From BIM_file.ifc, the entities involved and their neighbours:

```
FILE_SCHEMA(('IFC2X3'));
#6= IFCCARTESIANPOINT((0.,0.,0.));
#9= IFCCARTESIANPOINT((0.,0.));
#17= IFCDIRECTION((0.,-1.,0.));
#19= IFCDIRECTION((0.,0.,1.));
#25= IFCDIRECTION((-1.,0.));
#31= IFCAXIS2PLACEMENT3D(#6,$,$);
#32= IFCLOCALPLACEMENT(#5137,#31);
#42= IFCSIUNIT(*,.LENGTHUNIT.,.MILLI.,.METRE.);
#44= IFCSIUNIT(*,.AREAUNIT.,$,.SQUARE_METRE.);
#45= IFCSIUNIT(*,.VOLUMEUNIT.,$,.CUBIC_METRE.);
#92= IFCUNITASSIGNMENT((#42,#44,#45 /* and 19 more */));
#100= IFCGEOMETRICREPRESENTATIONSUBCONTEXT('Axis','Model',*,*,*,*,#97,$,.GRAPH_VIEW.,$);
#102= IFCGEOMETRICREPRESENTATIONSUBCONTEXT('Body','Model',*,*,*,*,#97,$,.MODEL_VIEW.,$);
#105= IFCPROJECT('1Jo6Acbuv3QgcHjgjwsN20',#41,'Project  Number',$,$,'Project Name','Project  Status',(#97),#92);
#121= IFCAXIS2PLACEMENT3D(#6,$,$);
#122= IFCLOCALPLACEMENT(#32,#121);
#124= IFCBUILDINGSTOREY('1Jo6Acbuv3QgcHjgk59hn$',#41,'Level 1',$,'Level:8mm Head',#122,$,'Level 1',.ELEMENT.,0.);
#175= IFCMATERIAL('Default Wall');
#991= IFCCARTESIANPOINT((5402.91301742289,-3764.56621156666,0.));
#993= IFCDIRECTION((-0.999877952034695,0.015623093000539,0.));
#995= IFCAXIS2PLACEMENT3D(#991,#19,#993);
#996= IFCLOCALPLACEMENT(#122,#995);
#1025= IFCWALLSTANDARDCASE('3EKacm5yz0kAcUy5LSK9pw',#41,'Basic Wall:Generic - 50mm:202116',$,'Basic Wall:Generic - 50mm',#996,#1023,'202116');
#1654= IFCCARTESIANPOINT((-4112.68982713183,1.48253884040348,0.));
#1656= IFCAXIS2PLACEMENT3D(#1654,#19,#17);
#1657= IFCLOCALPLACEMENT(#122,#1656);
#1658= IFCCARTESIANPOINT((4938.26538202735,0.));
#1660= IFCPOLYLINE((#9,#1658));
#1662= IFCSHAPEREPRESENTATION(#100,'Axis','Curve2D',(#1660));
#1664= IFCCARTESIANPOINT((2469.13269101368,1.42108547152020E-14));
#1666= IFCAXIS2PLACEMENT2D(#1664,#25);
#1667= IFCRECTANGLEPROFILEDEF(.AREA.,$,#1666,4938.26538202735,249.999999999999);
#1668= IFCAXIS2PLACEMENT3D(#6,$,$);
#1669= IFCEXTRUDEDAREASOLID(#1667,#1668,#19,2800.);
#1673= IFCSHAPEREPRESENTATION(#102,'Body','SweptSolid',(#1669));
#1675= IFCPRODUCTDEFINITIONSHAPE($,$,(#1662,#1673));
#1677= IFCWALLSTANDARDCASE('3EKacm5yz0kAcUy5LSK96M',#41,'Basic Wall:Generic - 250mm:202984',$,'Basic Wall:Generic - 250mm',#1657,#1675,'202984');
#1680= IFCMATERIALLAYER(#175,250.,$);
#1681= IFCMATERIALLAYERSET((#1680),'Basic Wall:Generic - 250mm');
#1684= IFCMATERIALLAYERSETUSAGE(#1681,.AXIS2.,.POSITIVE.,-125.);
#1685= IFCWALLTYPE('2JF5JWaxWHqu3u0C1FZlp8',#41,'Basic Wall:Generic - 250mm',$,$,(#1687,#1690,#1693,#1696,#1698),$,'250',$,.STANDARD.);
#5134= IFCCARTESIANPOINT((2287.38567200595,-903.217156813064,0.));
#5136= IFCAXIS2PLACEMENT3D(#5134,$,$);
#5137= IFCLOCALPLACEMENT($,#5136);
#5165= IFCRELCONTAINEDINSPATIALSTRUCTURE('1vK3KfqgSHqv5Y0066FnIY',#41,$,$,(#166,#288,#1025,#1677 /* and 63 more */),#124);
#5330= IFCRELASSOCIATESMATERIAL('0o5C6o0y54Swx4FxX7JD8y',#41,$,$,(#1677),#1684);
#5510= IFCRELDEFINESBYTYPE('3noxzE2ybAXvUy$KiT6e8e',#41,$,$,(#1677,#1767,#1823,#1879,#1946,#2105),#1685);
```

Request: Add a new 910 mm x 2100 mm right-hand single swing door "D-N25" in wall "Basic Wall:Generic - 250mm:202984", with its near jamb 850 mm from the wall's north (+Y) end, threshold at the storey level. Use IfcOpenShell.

```python
import numpy as np
import ifcopenshell
import ifcopenshell.api.feature
import ifcopenshell.api.geometry
import ifcopenshell.api.root
import ifcopenshell.api.spatial
import ifcopenshell.api.type
import ifcopenshell.geom
import ifcopenshell.util.element
import ifcopenshell.util.placement
import ifcopenshell.util.representation
import ifcopenshell.util.shape
import ifcopenshell.util.unit

model = ifcopenshell.open("BIM_file.ifc")
unit_scale = ifcopenshell.util.unit.calculate_unit_scale(model)
settings = ifcopenshell.geom.settings()


def volume(element):
    """Net volume in cubic metres, openings subtracted."""
    shape = ifcopenshell.geom.create_shape(settings, element)
    return ifcopenshell.util.shape.get_volume(shape.geometry)


wall = model.by_guid("3EKacm5yz0kAcUy5LSK96M")
storey = ifcopenshell.util.element.get_container(wall, ifc_class="IfcBuildingStorey")
context = ifcopenshell.util.representation.get_context(model, "Model", "Body", "MODEL_VIEW")
before = volume(wall)

width, height, from_end, sill = 0.91, 2.1, 0.85, 0.0  # metres

# The wall runs along its own X axis, and the end named is its -X end.
wall_shape = ifcopenshell.geom.create_shape(settings, wall)
x, y, z = ifcopenshell.util.shape.get_vertices(wall_shape.geometry).T
start = x.min() + from_end
face, thickness = float(y.min()), float(y.max() - y.min())
wall_matrix = ifcopenshell.util.placement.get_local_placement(wall.ObjectPlacement)
level = ifcopenshell.util.placement.get_local_placement(storey.ObjectPlacement)[2, 3]


def in_wall(x, y):
    """Placement at x, y metres in the wall's axes, at sill height."""
    matrix = wall_matrix.copy()
    matrix[:, 3] = wall_matrix @ np.array([x / unit_scale, y / unit_scale, 0.0, 1.0])
    matrix[2, 3] = level + sill / unit_scale
    return matrix


# Opening: a box that overshoots both wall faces by 50 mm.
opening = ifcopenshell.api.root.create_entity(model, ifc_class="IfcOpeningElement")
box = ifcopenshell.api.geometry.add_wall_representation(
    model, context=context, length=width, height=height, thickness=thickness + 0.1
)
ifcopenshell.api.geometry.assign_representation(model, product=opening, representation=box)
ifcopenshell.api.geometry.edit_object_placement(model, product=opening, matrix=in_wall(start, face - 0.05), is_si=False)
ifcopenshell.api.feature.add_feature(model, feature=opening, element=wall)

door = ifcopenshell.api.root.create_entity(model, ifc_class="IfcDoor", name="D-N25")
door.OverallWidth, door.OverallHeight = width / unit_scale, height / unit_scale
body = ifcopenshell.api.geometry.add_door_representation(
    model,
    context=context,
    overall_width=door.OverallWidth,
    overall_height=door.OverallHeight,
    operation_type="SINGLE_SWING_RIGHT",
    lining_properties={"LiningDepth": thickness / unit_scale, "ThresholdDepth": thickness / unit_scale},
)
ifcopenshell.api.geometry.assign_representation(model, product=door, representation=body)
ifcopenshell.api.spatial.assign_container(model, products=[door], relating_structure=storey)
fills = ifcopenshell.api.feature.add_filling(model, opening=opening, element=door)
fills.OwnerHistory = door.OwnerHistory  # required in IFC2X3

# IFC2X3 keeps the operation on the door style.
style = ifcopenshell.api.root.create_entity(model, ifc_class="IfcDoorStyle", name="D-N25")
style.OperationType, style.ConstructionType = "SINGLE_SWING_RIGHT", "NOTDEFINED"
style.ParameterTakesPrecedence = style.Sizeable = False
ifcopenshell.api.type.assign_type(model, related_objects=[door], relating_type=style)

# The lining spans the wall, so the door starts at the wall face.
ifcopenshell.api.geometry.edit_object_placement(model, product=door, matrix=in_wall(start, face), is_si=False)

after = volume(wall)

print(f"wall volume {before:.3f} -> {after:.3f} m3")

model.write("BIM_file_updated.ifc")
```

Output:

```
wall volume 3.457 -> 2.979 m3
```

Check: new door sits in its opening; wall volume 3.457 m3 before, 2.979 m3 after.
